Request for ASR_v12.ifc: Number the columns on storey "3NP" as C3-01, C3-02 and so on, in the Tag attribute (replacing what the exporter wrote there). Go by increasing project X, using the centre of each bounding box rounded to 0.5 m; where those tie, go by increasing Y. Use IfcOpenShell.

First a look at what the model holds.

```python
import ifcopenshell
import ifcopenshell.util.element
import ifcopenshell.util.placement

model = ifcopenshell.open("ASR_v12.ifc")
print(model.schema)
storey = next(s for s in model.by_type("IfcBuildingStorey") if s.Name == "3NP")
columns = [e for e in ifcopenshell.util.element.get_decomposition(storey) if e.is_a("IfcColumn")]
for e in sorted(columns, key=lambda e: e.id()):
    origin = ifcopenshell.util.placement.get_local_placement(e.ObjectPlacement)[:3, 3]
    print(e.id(), e.Tag, e.Name, origin.round(2) + 0.0, sep=" | ")
```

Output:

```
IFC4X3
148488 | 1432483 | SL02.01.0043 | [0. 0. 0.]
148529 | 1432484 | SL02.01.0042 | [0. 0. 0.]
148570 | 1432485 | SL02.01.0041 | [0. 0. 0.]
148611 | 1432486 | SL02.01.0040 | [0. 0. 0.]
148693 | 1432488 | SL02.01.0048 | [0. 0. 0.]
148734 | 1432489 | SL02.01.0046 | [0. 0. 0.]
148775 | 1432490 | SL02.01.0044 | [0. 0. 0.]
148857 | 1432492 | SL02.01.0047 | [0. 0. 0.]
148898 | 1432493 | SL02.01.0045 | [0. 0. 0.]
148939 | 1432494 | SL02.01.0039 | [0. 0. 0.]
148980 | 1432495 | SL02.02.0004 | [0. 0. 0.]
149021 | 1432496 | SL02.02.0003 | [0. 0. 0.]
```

```python
import ifcopenshell
import ifcopenshell.geom
import ifcopenshell.util.element
import ifcopenshell.util.shape

model = ifcopenshell.open("ASR_v12.ifc")
settings = ifcopenshell.geom.settings()
settings.set("use-world-coords", True)


def centre(element):
    shape = ifcopenshell.geom.create_shape(settings, element)
    return ifcopenshell.util.shape.get_bbox_centroid(shape.geometry)


storey = next(s for s in model.by_type("IfcBuildingStorey") if s.Name == "3NP")
columns = [e for e in ifcopenshell.util.element.get_decomposition(storey) if e.is_a("IfcColumn")]

# Insertion points can sit at a corner or the storey origin, so sort by the geometry (in metres).
centres = {e: centre(e) for e in columns}
columns.sort(key=lambda e: (round(centres[e][0] / 0.5), centres[e][1]))

for i, e in enumerate(columns, start=1):
    number = f"C3-{i:02d}"
    e.Tag = number
    print(e.id(), number)

model.write("ASR_v12_v2.ifc")
```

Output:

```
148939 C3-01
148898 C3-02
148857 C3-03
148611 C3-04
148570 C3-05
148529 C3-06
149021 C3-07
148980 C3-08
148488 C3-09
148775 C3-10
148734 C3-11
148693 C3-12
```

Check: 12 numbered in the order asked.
